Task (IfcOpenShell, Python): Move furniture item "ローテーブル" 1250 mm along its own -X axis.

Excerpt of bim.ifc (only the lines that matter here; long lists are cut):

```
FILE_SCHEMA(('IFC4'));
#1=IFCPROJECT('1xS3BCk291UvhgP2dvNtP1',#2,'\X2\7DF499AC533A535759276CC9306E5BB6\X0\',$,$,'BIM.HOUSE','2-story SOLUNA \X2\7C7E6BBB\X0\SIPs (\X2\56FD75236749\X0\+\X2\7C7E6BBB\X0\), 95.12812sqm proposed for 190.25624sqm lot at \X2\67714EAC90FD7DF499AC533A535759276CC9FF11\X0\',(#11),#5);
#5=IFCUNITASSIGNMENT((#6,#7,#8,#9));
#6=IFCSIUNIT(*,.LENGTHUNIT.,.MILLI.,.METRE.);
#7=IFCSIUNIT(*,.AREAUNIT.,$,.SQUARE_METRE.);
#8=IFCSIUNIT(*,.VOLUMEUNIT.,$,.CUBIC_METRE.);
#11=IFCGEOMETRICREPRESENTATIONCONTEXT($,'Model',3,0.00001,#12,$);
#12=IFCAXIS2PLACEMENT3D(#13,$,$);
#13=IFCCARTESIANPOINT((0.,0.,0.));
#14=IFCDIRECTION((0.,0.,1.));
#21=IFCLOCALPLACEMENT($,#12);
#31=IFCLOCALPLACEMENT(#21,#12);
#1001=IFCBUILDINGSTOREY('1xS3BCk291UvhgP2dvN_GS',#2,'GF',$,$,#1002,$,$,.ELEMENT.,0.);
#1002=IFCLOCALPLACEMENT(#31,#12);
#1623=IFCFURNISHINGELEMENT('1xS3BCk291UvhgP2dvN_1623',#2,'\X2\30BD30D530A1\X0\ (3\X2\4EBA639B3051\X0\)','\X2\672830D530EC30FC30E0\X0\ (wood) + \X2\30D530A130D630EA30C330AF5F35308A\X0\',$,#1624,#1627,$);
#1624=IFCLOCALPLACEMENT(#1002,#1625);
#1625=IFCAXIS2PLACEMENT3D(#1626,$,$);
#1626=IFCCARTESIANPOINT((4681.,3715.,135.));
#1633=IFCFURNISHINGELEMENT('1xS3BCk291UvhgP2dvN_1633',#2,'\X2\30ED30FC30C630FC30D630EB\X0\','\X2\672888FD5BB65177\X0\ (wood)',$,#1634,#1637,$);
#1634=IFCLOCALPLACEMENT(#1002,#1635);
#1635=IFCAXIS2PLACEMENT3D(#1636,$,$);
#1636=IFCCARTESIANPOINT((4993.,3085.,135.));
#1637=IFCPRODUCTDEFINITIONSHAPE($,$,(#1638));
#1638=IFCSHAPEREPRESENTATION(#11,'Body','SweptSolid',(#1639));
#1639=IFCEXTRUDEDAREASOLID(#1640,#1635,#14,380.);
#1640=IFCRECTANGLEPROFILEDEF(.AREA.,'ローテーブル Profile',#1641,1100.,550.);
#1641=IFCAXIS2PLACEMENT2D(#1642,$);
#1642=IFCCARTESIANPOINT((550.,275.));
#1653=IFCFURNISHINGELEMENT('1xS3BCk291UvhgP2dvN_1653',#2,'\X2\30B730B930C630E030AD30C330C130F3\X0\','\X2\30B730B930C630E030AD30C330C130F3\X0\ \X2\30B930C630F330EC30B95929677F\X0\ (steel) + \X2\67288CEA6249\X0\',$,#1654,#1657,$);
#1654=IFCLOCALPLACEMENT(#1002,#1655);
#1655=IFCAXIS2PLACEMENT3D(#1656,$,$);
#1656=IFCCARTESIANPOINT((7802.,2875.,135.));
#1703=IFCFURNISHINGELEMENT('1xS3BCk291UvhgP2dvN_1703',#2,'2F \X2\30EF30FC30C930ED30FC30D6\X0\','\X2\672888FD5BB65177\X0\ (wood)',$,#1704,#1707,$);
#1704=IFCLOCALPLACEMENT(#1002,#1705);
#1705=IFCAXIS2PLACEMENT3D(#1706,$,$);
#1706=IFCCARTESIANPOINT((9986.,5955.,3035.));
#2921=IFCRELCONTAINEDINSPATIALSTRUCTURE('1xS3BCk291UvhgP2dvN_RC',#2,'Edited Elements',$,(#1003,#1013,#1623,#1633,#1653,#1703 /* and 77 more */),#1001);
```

```python
import ifcopenshell
import ifcopenshell.api.geometry
import ifcopenshell.util.placement
import ifcopenshell.util.unit

model = ifcopenshell.open("bim.ifc")
unit_scale = ifcopenshell.util.unit.calculate_unit_scale(model)

item = model.by_id(1633)
matrix = ifcopenshell.util.placement.get_local_placement(item.ObjectPlacement)
matrix[:3, 3] -= matrix[:3, 0] * 1.25 / unit_scale
ifcopenshell.api.geometry.edit_object_placement(model, product=item, matrix=matrix, is_si=False)

print(ifcopenshell.util.placement.get_local_placement(item.ObjectPlacement).round(3) + 0.0)

model.write("bim_rev.ifc")
```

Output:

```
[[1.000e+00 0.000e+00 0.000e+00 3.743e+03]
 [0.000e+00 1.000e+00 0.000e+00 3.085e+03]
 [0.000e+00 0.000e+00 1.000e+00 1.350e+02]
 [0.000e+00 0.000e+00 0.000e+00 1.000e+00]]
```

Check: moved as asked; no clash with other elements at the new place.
